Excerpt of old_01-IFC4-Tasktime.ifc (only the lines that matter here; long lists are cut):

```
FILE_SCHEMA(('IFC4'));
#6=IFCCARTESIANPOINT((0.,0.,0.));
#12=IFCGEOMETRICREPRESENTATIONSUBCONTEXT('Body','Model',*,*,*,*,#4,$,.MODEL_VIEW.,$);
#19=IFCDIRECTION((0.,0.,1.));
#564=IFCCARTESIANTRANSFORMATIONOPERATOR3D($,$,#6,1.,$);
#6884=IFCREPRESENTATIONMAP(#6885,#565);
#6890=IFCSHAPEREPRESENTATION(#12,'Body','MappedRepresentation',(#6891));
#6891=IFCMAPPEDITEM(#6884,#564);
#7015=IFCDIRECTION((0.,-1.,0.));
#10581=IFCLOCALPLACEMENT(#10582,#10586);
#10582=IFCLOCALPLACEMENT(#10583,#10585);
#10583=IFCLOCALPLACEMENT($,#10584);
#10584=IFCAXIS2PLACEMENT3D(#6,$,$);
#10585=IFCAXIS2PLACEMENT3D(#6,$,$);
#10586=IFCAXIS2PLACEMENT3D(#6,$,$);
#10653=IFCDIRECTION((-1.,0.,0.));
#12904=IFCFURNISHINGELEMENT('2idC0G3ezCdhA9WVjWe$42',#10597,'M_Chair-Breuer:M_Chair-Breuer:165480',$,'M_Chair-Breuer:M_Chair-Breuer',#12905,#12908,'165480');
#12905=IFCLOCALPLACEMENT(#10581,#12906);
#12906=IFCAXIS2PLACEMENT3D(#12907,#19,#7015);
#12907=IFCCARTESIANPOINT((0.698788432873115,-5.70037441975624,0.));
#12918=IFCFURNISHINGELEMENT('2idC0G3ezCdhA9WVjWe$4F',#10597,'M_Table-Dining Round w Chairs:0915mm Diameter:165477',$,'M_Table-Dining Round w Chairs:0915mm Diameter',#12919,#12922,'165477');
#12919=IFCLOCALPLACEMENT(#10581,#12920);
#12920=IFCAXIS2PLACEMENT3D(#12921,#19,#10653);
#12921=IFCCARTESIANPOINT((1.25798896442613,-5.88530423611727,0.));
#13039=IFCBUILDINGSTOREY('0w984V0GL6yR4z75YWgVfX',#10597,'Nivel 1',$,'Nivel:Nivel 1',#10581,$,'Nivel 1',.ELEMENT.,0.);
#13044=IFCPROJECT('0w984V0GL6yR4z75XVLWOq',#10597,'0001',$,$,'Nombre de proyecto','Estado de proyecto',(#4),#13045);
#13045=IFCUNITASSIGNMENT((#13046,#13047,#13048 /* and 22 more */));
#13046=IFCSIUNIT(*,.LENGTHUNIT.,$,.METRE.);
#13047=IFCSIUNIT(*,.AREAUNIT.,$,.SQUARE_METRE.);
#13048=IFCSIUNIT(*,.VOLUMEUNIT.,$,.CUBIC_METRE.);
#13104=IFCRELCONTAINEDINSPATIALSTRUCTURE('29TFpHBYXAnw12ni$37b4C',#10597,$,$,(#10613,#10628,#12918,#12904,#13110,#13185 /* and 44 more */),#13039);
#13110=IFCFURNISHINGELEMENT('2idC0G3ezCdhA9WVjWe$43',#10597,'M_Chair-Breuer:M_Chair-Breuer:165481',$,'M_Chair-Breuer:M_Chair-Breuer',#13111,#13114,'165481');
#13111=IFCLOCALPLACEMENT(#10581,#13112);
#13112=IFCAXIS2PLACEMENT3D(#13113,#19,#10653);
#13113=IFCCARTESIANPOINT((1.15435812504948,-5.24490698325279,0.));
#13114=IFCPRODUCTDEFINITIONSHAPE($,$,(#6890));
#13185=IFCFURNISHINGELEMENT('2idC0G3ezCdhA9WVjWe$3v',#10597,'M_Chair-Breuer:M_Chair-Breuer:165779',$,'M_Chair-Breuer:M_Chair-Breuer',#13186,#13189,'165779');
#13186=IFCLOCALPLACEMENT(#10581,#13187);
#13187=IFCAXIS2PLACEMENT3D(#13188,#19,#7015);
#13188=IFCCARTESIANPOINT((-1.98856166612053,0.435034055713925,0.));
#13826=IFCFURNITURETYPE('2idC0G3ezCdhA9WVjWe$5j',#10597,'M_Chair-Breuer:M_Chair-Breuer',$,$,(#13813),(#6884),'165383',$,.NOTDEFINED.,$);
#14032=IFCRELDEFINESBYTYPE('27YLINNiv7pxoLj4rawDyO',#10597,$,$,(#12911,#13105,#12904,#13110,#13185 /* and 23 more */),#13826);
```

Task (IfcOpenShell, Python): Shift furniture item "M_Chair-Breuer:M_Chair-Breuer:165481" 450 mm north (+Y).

```python
import ifcopenshell
import ifcopenshell.api.geometry
import ifcopenshell.util.placement
import ifcopenshell.util.unit

model = ifcopenshell.open("old_01-IFC4-Tasktime.ifc")
unit_scale = ifcopenshell.util.unit.calculate_unit_scale(model)

item = model.by_guid("2idC0G3ezCdhA9WVjWe$43")
matrix = ifcopenshell.util.placement.get_local_placement(item.ObjectPlacement)
matrix[1, 3] += 0.45 / unit_scale
ifcopenshell.api.geometry.edit_object_placement(model, product=item, matrix=matrix, is_si=False)

print(ifcopenshell.util.placement.get_local_placement(item.ObjectPlacement).round(3) + 0.0)

model.write("old_01-IFC4-Tasktime_edited.ifc")
```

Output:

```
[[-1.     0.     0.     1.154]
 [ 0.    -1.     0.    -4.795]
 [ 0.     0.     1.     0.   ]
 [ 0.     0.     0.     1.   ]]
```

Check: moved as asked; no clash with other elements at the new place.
